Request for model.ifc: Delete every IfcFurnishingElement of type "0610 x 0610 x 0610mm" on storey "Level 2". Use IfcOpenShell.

First a look at what the model holds.

```python
import ifcopenshell
import ifcopenshell.util.element

model = ifcopenshell.open("model.ifc")
print(model.schema)
storey = next(s for s in model.by_type("IfcBuildingStorey") if s.Name == "Level 2")
furniture = [e for e in ifcopenshell.util.element.get_decomposition(storey) if e.is_a("IfcFurnishingElement")]
seen = {}
for e in furniture:
    element_type = ifcopenshell.util.element.get_type(e)
    name = element_type.Name if element_type not in (None, e) else None
    seen[name] = seen.get(name, 0) + 1
for name, count in sorted(seen.items(), key=str):
    print(count, "x", name)
```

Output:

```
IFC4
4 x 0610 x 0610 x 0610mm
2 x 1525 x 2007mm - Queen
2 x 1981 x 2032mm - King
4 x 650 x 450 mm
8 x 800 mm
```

```python
import ifcopenshell
import ifcopenshell.api.root
import ifcopenshell.util.element

model = ifcopenshell.open("model.ifc")

storey = next(s for s in model.by_type("IfcBuildingStorey") if s.Name == "Level 2")
furniture = [e for e in ifcopenshell.util.element.get_decomposition(storey) if e.is_a("IfcFurnishingElement")]
targets = [e for e in furniture if (t := ifcopenshell.util.element.get_type(e)) not in (None, e) and t.Name == "0610 x 0610 x 0610mm"]

for e in targets:
    ifcopenshell.api.root.remove_product(model, product=e)
print(len(targets), "removed")

model.write("model_updated.ifc")
```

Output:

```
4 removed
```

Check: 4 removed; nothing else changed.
